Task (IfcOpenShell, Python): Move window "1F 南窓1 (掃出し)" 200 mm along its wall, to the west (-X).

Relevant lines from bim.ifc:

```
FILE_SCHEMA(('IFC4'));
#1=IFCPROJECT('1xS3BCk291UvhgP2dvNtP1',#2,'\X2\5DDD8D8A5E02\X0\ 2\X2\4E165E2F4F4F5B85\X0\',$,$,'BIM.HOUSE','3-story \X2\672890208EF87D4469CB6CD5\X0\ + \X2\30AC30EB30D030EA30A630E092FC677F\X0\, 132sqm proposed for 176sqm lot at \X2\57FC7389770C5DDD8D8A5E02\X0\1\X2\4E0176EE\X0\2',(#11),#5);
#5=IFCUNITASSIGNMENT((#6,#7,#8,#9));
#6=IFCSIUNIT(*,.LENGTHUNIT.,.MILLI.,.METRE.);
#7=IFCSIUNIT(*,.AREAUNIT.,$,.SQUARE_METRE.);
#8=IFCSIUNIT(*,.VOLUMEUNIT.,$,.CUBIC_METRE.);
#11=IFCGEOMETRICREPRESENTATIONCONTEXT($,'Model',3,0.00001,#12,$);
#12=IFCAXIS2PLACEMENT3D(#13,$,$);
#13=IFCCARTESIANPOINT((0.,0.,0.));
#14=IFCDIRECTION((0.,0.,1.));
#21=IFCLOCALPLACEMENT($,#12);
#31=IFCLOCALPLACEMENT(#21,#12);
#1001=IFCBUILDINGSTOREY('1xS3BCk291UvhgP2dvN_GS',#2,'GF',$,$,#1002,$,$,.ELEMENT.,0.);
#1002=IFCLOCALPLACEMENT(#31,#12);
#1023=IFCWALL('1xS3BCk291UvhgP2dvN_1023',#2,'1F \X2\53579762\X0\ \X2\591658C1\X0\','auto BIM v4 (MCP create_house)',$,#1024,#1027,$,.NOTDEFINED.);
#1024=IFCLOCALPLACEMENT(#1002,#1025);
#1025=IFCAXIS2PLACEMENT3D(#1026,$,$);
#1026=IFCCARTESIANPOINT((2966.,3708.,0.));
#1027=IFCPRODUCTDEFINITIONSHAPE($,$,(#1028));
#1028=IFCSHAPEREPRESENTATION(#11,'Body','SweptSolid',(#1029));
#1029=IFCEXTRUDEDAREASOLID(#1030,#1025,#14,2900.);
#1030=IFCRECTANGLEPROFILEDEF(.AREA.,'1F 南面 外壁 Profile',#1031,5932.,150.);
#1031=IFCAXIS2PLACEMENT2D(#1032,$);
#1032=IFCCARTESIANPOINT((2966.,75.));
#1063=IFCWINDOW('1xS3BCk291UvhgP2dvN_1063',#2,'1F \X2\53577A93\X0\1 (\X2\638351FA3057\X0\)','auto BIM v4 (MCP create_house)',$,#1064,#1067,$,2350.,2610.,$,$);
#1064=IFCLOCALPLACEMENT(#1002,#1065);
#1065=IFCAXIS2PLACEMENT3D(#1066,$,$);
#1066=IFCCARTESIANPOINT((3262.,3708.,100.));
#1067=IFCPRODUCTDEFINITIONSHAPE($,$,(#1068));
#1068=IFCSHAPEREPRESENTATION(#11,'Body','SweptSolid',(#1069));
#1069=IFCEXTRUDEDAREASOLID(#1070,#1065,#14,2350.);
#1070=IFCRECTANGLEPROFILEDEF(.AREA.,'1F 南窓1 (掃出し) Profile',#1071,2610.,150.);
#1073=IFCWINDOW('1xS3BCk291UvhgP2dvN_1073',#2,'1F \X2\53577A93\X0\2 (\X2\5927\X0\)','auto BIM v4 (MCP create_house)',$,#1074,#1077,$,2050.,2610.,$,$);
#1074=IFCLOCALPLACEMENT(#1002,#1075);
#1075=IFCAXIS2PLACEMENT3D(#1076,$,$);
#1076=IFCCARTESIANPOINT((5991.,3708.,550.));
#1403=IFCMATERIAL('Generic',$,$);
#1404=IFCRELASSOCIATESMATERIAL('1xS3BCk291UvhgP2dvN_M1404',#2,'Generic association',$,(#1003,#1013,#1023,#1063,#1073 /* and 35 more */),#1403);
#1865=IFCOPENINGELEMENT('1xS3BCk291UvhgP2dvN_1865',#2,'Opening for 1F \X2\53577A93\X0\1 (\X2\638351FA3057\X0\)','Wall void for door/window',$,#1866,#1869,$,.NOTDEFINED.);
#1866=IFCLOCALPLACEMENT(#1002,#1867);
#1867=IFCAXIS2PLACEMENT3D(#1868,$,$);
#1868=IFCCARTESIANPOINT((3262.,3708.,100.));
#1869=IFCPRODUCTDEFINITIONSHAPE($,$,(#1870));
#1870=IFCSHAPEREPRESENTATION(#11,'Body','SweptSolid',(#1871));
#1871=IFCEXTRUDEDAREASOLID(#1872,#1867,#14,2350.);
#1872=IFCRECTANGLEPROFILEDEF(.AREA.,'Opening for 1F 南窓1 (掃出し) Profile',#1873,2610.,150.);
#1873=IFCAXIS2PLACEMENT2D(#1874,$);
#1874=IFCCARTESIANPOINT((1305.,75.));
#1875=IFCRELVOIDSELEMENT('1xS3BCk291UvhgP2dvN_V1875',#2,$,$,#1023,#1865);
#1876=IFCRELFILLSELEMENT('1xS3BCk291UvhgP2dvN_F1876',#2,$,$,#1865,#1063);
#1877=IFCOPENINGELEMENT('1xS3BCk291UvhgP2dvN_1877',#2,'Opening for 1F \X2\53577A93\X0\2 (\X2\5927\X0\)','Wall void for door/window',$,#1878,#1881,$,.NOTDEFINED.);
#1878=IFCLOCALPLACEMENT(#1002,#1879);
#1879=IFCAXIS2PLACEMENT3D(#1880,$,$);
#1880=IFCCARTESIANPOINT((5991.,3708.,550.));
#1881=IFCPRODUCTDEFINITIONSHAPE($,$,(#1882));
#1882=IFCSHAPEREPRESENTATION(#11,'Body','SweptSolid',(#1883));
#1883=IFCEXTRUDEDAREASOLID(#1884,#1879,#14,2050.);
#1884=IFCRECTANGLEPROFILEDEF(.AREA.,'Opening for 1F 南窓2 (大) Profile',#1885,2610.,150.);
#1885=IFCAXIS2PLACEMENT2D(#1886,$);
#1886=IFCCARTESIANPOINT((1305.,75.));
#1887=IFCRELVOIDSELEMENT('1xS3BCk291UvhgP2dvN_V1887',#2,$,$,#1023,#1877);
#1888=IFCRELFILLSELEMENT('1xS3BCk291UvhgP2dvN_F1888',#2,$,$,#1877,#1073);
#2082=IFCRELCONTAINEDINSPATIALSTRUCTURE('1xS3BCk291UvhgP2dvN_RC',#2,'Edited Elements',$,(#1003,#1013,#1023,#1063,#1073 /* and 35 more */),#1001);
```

```python
import ifcopenshell
import ifcopenshell.api.geometry
import ifcopenshell.util.placement
import ifcopenshell.util.unit

model = ifcopenshell.open("bim.ifc")
unit_scale = ifcopenshell.util.unit.calculate_unit_scale(model)

window = model.by_guid("1xS3BCk291UvhgP2dvN_1063")
opening = window.FillsVoids[0].RelatingOpeningElement
wall = opening.VoidsElements[0].RelatingBuildingElement

wall_matrix = ifcopenshell.util.placement.get_local_placement(wall.ObjectPlacement)
shift = wall_matrix[:3, 0] * -0.2 / unit_scale
before = ifcopenshell.util.placement.get_local_placement(window.ObjectPlacement)[:3, 3].copy()

# The window is not placed relative to its opening, so move both.
for product in (opening, window):
    matrix = ifcopenshell.util.placement.get_local_placement(product.ObjectPlacement)
    matrix[:3, 3] += shift
    ifcopenshell.api.geometry.edit_object_placement(model, product=product, matrix=matrix, is_si=False)

after = ifcopenshell.util.placement.get_local_placement(window.ObjectPlacement)[:3, 3]
print("window moved by", (after - before).round(3) + 0.0)

model.write("bim_v2.ifc")
```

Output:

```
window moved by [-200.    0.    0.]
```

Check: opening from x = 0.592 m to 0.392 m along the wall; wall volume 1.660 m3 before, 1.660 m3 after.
